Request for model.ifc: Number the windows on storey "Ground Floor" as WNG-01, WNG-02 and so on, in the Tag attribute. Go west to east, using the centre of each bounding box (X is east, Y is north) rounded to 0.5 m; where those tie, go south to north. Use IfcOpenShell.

First a look at what the model holds.

```python
import ifcopenshell
import ifcopenshell.util.element
import ifcopenshell.util.placement

model = ifcopenshell.open("model.ifc")
print(model.schema)
storey = next(s for s in model.by_type("IfcBuildingStorey") if s.Name == "Ground Floor")
windows = [e for e in ifcopenshell.util.element.get_decomposition(storey) if e.is_a("IfcWindow")]
for e in sorted(windows, key=lambda e: e.id()):
    origin = ifcopenshell.util.placement.get_local_placement(e.ObjectPlacement)[:3, 3]
    print(e.id(), e.Tag, e.Name, origin.round(2) + 0.0, sep=" | ")
```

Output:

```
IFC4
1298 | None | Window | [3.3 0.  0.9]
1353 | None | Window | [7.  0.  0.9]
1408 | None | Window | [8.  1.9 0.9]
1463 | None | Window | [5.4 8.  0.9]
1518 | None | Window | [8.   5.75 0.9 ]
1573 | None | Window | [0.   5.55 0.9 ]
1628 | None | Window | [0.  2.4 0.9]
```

```python
import ifcopenshell
import ifcopenshell.geom
import ifcopenshell.util.element
import ifcopenshell.util.shape

model = ifcopenshell.open("model.ifc")
settings = ifcopenshell.geom.settings()
settings.set("use-world-coords", True)


def centre(element):
    shape = ifcopenshell.geom.create_shape(settings, element)
    return ifcopenshell.util.shape.get_bbox_centroid(shape.geometry)


storey = next(s for s in model.by_type("IfcBuildingStorey") if s.Name == "Ground Floor")
windows = [e for e in ifcopenshell.util.element.get_decomposition(storey) if e.is_a("IfcWindow")]

# Insertion points can sit at a corner or the storey origin, so sort by the geometry (in metres).
centres = {e: centre(e) for e in windows}
windows.sort(key=lambda e: (round(centres[e][0] / 0.5), centres[e][1]))

for i, e in enumerate(windows, start=1):
    number = f"WNG-{i:02d}"
    e.Tag = number
    print(e.id(), number)

model.write("model_v2.ifc")
```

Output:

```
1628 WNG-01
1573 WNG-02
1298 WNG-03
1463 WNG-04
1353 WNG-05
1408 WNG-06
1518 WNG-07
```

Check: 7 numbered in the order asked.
